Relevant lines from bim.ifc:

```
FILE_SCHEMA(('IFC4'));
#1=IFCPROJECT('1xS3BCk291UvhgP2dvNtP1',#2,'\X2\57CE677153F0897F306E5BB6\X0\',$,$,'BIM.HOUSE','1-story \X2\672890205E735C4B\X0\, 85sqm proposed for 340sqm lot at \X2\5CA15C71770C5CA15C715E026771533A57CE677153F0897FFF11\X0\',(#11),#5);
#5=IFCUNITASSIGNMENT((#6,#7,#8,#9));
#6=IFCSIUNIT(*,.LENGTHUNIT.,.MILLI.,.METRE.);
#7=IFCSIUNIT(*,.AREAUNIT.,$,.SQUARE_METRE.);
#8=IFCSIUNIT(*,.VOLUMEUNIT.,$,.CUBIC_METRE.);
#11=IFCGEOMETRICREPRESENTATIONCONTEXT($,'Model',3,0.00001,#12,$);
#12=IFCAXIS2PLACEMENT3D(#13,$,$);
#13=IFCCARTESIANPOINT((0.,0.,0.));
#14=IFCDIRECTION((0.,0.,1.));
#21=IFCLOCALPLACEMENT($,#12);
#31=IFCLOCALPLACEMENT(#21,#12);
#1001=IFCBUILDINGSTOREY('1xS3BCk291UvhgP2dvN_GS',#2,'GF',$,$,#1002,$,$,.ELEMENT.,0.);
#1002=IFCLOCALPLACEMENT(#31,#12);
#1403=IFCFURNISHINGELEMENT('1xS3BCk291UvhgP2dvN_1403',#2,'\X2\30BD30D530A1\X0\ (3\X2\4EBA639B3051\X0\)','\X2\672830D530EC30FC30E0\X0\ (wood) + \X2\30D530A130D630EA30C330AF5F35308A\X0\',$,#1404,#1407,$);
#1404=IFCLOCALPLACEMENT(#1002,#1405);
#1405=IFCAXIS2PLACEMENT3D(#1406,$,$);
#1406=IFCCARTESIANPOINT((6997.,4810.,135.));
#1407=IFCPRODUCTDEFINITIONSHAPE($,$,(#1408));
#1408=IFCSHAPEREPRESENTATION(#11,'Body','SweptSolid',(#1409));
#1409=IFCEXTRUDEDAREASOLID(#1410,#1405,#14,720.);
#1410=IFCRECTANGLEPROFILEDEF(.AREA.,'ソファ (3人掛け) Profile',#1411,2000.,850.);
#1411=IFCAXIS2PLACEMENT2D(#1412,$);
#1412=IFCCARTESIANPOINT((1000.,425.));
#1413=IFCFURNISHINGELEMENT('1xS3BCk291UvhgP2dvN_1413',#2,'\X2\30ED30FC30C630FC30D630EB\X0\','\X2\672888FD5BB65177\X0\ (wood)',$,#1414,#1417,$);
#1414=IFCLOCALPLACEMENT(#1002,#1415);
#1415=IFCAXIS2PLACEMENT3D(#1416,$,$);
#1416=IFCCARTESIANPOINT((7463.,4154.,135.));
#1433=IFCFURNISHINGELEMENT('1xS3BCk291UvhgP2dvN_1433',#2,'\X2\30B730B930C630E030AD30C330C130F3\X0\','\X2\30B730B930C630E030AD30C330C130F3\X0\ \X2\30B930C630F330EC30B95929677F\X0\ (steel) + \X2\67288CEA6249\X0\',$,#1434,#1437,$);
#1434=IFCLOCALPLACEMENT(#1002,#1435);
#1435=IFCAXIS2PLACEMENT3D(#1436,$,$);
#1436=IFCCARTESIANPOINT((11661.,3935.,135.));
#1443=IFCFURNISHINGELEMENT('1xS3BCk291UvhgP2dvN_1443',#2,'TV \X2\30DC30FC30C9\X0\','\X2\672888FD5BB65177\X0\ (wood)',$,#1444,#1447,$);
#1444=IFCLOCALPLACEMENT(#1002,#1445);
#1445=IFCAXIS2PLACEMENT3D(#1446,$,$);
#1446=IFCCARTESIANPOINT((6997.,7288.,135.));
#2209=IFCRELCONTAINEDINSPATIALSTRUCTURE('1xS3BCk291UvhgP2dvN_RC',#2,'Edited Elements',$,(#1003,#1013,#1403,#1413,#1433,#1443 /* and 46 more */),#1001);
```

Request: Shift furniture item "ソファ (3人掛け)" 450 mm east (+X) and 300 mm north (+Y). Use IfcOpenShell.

```python
import ifcopenshell
import ifcopenshell.api.geometry
import ifcopenshell.util.placement

model = ifcopenshell.open("bim.ifc")

item = model.by_guid("1xS3BCk291UvhgP2dvN_1403")
matrix = ifcopenshell.util.placement.get_local_placement(item.ObjectPlacement)
matrix[0, 3] += 450.0
matrix[1, 3] += 300.0
ifcopenshell.api.geometry.edit_object_placement(model, product=item, matrix=matrix, is_si=False)

print(ifcopenshell.util.placement.get_local_placement(item.ObjectPlacement).round(3) + 0.0)

model.write("bim_v2.ifc")
```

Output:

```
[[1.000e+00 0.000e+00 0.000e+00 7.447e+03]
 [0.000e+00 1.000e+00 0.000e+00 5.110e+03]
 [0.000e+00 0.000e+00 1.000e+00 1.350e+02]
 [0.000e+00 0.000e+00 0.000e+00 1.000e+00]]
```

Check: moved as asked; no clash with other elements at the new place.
